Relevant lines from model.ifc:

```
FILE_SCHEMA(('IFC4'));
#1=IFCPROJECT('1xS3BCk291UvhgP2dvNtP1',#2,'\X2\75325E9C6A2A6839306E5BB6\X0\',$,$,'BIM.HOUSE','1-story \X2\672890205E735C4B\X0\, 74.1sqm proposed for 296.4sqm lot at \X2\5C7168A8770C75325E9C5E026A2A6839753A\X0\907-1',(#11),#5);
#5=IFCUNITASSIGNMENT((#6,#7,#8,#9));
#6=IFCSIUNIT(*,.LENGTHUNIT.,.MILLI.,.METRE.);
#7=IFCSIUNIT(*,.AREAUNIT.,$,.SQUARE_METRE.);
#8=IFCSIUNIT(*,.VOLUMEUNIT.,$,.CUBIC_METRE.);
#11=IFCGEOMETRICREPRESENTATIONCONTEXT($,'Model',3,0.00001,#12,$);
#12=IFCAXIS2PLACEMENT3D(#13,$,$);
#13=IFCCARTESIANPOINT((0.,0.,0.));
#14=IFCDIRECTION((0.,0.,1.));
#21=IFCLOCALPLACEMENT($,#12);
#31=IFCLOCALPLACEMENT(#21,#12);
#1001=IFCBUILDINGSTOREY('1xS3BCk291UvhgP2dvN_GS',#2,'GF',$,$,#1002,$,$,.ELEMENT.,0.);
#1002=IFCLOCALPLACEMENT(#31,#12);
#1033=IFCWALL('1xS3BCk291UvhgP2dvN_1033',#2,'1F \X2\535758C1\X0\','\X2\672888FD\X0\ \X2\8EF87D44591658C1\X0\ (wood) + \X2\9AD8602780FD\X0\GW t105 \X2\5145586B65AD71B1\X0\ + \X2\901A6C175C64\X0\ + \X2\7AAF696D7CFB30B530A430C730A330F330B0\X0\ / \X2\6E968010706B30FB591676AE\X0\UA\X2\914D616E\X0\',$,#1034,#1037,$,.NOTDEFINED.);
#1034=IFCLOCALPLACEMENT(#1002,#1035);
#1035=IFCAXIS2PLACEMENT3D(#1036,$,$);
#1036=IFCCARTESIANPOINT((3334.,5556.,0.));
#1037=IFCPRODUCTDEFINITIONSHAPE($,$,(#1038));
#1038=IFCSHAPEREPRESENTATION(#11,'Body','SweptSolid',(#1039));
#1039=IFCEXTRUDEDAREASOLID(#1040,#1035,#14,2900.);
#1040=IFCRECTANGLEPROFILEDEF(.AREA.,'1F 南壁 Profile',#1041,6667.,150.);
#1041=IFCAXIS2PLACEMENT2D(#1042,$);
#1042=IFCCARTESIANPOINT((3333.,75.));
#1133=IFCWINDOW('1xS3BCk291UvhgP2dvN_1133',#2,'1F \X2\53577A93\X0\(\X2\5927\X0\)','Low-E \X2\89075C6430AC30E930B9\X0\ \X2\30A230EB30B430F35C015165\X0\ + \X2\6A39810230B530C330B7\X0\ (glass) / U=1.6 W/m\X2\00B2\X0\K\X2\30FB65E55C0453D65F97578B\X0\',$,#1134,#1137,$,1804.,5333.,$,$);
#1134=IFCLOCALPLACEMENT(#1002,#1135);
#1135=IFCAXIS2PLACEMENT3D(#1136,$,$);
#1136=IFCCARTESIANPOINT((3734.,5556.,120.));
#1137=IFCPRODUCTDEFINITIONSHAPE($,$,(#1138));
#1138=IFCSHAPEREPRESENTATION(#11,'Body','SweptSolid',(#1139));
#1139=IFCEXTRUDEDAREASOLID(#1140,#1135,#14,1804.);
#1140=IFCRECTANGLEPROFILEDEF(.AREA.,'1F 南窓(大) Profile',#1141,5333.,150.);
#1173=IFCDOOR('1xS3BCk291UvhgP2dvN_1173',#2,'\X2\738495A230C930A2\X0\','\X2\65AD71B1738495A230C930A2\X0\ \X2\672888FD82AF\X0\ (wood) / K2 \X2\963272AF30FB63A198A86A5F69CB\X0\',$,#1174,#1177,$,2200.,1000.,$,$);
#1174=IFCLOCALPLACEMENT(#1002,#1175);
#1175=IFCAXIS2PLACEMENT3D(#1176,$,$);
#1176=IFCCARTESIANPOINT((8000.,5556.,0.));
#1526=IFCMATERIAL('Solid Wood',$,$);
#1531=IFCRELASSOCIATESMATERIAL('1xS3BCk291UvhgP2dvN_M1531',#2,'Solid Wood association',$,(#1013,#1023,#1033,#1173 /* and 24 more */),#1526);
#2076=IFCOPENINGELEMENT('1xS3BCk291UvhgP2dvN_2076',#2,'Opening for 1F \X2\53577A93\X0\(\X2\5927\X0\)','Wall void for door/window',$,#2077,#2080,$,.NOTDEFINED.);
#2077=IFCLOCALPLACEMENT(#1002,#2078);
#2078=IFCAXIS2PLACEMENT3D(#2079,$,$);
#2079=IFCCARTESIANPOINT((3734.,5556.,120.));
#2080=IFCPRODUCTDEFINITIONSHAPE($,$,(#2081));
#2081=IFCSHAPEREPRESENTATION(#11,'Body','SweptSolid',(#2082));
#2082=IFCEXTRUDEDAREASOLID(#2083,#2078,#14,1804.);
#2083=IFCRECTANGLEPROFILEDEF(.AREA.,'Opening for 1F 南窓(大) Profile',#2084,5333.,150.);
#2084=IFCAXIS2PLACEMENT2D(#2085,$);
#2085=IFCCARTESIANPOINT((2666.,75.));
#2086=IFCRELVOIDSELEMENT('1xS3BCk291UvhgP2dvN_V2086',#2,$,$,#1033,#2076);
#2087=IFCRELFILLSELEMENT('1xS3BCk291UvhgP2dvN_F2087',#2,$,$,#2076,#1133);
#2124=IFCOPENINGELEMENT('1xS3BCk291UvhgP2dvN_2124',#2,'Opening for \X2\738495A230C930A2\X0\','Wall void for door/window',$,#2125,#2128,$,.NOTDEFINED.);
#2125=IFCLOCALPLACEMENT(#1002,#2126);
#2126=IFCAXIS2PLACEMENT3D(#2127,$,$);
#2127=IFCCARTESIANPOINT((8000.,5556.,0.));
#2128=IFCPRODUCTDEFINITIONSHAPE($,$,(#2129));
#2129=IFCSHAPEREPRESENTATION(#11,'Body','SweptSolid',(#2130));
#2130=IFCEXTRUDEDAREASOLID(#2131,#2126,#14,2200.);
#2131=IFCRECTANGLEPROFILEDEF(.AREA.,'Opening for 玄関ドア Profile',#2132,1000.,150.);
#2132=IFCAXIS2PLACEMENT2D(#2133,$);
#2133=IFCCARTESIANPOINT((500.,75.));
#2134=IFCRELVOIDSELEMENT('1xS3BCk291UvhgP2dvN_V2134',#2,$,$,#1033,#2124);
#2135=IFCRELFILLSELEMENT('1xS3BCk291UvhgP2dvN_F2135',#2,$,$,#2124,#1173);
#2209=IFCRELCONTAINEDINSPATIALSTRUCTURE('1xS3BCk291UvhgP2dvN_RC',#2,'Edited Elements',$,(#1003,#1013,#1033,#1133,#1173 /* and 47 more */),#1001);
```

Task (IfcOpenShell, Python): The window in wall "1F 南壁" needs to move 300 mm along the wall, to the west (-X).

```python
import ifcopenshell
import ifcopenshell.api.geometry
import ifcopenshell.util.placement
import ifcopenshell.util.unit

model = ifcopenshell.open("model.ifc")
unit_scale = ifcopenshell.util.unit.calculate_unit_scale(model)

window = model.by_guid("1xS3BCk291UvhgP2dvN_1133")
opening = window.FillsVoids[0].RelatingOpeningElement
wall = opening.VoidsElements[0].RelatingBuildingElement

wall_matrix = ifcopenshell.util.placement.get_local_placement(wall.ObjectPlacement)
shift = wall_matrix[:3, 0] * -0.3 / unit_scale
before = ifcopenshell.util.placement.get_local_placement(window.ObjectPlacement)[:3, 3].copy()

# The window is not placed relative to its opening, so move both.
for product in (opening, window):
    matrix = ifcopenshell.util.placement.get_local_placement(product.ObjectPlacement)
    matrix[:3, 3] += shift
    ifcopenshell.api.geometry.edit_object_placement(model, product=product, matrix=matrix, is_si=False)

after = ifcopenshell.util.placement.get_local_placement(window.ObjectPlacement)[:3, 3]
print("window moved by", (after - before).round(3) + 0.0)

model.write("model_edited.ifc")
```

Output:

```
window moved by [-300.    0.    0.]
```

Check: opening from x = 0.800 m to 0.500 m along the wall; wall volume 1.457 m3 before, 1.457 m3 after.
